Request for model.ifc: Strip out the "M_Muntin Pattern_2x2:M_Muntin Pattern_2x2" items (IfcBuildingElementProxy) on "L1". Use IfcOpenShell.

First a look at what the model holds.

```python
import ifcopenshell
import ifcopenshell.util.element

model = ifcopenshell.open("model.ifc")
print(model.schema)
storey = next(s for s in model.by_type("IfcBuildingStorey") if s.Name == "L1")
proxies = [e for e in ifcopenshell.util.element.get_decomposition(storey) if e.is_a("IfcBuildingElementProxy")]
seen = {}
for e in proxies:
    element_type = ifcopenshell.util.element.get_type(e)
    name = element_type.Name if element_type not in (None, e) else None
    seen[name] = seen.get(name, 0) + 1
for name, count in sorted(seen.items(), key=str):
    print(count, "x", name)
```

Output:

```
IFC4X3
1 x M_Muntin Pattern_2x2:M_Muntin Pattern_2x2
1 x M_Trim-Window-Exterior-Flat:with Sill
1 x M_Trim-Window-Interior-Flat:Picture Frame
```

```python
import ifcopenshell
import ifcopenshell.api.root
import ifcopenshell.util.element

model = ifcopenshell.open("model.ifc")

storey = next(s for s in model.by_type("IfcBuildingStorey") if s.Name == "L1")
proxies = [e for e in ifcopenshell.util.element.get_decomposition(storey) if e.is_a("IfcBuildingElementProxy")]
targets = [e for e in proxies if (t := ifcopenshell.util.element.get_type(e)) not in (None, e) and t.Name == "M_Muntin Pattern_2x2:M_Muntin Pattern_2x2"]

for e in targets:
    ifcopenshell.api.root.remove_product(model, product=e)
print(len(targets), "removed")

model.write("model_v2.ifc")
```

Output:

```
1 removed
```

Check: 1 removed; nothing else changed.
